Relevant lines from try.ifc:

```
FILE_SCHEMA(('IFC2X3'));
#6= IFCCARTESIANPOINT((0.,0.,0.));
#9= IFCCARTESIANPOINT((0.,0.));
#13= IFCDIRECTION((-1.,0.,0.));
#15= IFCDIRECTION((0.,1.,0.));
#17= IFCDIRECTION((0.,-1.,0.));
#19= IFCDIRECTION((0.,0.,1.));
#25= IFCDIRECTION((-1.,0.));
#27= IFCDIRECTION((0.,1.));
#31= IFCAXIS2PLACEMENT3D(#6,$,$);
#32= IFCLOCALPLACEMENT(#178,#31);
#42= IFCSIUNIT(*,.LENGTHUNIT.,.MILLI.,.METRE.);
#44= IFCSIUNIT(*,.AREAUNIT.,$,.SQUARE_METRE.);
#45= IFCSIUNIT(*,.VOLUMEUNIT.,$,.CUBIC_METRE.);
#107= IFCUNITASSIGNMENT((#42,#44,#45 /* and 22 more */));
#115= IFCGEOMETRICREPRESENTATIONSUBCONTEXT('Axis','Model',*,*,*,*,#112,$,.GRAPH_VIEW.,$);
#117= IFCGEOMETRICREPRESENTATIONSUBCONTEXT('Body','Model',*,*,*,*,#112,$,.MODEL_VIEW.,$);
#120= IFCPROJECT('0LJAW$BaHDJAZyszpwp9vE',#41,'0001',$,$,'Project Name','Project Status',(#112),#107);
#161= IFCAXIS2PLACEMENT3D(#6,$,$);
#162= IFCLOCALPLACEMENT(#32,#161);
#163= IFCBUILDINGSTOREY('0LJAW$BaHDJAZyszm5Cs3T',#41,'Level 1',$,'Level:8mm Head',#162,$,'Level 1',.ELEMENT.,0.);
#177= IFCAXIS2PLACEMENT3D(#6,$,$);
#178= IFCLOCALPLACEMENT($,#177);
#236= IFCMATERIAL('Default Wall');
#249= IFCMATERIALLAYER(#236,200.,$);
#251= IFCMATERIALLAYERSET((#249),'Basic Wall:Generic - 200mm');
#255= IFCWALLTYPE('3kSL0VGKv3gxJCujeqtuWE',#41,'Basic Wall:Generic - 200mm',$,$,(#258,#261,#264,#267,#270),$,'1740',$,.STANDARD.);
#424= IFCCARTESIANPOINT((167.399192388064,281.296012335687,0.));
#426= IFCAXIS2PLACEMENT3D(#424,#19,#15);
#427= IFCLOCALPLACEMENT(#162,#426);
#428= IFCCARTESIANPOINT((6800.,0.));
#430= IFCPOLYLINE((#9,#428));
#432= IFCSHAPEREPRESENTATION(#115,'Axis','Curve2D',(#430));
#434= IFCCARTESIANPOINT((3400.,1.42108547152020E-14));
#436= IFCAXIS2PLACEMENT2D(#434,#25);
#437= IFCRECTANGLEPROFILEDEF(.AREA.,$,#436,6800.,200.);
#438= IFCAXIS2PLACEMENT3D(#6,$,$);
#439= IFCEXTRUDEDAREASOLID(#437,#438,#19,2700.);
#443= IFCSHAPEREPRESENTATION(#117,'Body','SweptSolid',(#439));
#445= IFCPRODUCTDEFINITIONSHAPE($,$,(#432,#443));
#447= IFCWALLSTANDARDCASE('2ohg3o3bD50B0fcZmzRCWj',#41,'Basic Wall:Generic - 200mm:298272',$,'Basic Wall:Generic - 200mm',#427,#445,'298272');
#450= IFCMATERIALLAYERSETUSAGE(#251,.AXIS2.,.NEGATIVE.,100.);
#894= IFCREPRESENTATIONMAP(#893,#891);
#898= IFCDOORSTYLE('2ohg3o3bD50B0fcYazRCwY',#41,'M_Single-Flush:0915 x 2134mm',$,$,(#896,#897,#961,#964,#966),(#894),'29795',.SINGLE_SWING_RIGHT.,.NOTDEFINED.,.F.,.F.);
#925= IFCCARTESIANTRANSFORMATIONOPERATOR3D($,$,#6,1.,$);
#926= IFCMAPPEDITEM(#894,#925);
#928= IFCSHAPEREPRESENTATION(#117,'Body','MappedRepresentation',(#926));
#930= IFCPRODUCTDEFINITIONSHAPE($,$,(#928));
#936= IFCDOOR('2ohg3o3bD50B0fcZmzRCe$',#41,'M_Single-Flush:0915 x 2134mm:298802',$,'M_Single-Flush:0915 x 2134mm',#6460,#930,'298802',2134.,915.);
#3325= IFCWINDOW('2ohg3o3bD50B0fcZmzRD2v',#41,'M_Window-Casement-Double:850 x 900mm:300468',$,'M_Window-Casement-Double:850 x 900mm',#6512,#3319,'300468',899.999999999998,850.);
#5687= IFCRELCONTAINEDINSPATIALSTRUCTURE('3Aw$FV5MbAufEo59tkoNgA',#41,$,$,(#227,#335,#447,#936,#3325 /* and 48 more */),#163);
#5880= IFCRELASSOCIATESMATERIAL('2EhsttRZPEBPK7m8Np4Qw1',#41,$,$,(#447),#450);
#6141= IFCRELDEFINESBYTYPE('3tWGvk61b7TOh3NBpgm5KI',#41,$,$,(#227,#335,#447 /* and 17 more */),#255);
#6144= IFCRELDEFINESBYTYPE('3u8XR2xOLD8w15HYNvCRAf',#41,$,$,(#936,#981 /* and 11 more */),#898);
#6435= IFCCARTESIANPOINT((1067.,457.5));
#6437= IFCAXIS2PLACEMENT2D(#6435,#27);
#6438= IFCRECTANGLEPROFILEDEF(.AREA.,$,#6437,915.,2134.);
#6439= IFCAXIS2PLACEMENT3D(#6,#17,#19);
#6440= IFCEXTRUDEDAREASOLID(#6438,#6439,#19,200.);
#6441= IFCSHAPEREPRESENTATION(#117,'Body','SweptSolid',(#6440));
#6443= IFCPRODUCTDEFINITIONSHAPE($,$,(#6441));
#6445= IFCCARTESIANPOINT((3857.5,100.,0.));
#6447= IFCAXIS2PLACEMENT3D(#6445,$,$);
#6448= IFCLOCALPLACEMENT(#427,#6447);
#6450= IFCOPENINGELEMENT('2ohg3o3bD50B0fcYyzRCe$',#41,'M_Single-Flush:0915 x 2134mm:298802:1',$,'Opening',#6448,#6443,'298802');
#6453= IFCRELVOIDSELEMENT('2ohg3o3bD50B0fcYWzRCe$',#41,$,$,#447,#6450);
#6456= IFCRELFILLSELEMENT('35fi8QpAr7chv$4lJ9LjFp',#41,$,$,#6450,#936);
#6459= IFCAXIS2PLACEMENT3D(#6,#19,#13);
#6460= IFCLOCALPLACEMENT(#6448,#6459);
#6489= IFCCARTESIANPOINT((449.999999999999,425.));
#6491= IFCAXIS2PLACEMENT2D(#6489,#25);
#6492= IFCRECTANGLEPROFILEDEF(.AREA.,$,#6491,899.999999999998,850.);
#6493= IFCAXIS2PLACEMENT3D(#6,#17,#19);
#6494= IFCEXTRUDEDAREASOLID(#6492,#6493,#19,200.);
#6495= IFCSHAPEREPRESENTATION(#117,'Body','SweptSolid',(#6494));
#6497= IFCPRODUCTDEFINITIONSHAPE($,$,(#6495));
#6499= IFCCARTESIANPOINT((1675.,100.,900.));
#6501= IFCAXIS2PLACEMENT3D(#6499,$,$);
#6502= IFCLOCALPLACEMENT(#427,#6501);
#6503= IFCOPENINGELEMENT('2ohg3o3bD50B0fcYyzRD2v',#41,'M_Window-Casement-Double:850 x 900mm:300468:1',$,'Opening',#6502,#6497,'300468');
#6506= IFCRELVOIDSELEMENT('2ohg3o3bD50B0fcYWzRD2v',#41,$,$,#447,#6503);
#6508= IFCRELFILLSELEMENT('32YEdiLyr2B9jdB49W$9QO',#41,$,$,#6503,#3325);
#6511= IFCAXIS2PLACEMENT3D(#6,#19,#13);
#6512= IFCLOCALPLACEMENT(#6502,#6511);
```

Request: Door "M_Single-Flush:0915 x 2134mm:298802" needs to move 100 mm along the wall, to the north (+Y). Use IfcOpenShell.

```python
import ifcopenshell
import ifcopenshell.api.geometry
import ifcopenshell.util.placement
import ifcopenshell.util.unit

model = ifcopenshell.open("try.ifc")
unit_scale = ifcopenshell.util.unit.calculate_unit_scale(model)

door = model.by_guid("2ohg3o3bD50B0fcZmzRCe$")
opening = door.FillsVoids[0].RelatingOpeningElement
wall = opening.VoidsElements[0].RelatingBuildingElement

wall_matrix = ifcopenshell.util.placement.get_local_placement(wall.ObjectPlacement)
shift = wall_matrix[:3, 0] * 0.1 / unit_scale
before = ifcopenshell.util.placement.get_local_placement(door.ObjectPlacement)[:3, 3].copy()

# The door is placed relative to its opening, so it follows when the opening moves.
matrix = ifcopenshell.util.placement.get_local_placement(opening.ObjectPlacement)
matrix[:3, 3] += shift
ifcopenshell.api.geometry.edit_object_placement(
    model, product=opening, matrix=matrix, is_si=False, should_transform_children=True
)

after = ifcopenshell.util.placement.get_local_placement(door.ObjectPlacement)[:3, 3]
print("door moved by", (after - before).round(3) + 0.0)

model.write("try_updated.ifc")
```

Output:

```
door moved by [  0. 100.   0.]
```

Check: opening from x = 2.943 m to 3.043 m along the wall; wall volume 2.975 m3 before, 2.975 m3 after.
